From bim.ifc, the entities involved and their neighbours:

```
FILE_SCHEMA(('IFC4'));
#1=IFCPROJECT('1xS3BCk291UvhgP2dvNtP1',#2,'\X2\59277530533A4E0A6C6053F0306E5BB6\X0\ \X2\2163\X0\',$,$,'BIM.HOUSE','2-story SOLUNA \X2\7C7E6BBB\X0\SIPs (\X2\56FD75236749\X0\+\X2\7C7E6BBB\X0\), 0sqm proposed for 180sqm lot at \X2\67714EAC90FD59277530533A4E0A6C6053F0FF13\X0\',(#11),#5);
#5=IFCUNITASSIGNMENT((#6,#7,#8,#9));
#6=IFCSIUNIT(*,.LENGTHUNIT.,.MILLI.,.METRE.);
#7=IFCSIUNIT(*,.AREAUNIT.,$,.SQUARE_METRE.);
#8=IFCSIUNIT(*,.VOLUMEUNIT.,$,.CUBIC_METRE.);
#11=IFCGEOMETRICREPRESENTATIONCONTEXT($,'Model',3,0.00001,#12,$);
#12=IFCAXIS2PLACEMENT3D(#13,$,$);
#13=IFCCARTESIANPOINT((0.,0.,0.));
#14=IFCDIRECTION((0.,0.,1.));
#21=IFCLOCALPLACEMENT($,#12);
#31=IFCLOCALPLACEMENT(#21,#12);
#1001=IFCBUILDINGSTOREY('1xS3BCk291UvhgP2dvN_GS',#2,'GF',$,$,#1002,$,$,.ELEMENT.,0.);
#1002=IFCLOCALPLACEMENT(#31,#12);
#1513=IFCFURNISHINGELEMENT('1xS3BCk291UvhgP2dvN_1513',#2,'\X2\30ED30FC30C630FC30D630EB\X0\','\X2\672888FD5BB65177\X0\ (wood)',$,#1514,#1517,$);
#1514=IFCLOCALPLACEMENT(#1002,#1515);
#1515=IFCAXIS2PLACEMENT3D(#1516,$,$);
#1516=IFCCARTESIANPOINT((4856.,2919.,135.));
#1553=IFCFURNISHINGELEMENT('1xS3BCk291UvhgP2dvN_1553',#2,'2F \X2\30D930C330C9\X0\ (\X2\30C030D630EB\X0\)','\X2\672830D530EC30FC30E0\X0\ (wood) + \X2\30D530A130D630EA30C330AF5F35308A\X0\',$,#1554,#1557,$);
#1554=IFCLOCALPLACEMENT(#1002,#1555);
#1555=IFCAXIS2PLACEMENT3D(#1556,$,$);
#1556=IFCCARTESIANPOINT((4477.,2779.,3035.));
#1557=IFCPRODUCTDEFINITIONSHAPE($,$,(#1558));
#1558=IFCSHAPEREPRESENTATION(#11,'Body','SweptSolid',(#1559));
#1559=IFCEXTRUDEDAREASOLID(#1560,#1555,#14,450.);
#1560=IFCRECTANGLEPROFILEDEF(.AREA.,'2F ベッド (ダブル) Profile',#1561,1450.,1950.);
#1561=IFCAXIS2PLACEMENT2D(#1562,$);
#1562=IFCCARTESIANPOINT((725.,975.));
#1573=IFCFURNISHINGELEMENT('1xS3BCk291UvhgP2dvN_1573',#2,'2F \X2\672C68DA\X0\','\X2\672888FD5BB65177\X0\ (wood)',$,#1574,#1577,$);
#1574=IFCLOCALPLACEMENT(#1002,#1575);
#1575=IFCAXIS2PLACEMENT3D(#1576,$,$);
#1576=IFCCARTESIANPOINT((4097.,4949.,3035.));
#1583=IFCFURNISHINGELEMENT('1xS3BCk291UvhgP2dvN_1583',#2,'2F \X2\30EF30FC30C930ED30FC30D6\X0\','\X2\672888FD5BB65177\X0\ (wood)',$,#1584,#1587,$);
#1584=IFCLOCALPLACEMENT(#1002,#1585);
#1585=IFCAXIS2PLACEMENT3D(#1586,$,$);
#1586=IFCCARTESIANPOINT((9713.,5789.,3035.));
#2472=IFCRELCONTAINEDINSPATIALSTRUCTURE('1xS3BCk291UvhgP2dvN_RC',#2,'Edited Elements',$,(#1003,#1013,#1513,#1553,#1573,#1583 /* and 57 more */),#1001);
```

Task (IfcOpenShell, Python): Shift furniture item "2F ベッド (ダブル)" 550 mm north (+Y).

```python
import ifcopenshell
import ifcopenshell.api.geometry
import ifcopenshell.util.placement
import ifcopenshell.util.unit

model = ifcopenshell.open("bim.ifc")
unit_scale = ifcopenshell.util.unit.calculate_unit_scale(model)

item = model.by_guid("1xS3BCk291UvhgP2dvN_1553")
matrix = ifcopenshell.util.placement.get_local_placement(item.ObjectPlacement)
matrix[1, 3] += 0.55 / unit_scale
ifcopenshell.api.geometry.edit_object_placement(model, product=item, matrix=matrix, is_si=False)

print(ifcopenshell.util.placement.get_local_placement(item.ObjectPlacement).round(3) + 0.0)

model.write("bim_updated.ifc")
```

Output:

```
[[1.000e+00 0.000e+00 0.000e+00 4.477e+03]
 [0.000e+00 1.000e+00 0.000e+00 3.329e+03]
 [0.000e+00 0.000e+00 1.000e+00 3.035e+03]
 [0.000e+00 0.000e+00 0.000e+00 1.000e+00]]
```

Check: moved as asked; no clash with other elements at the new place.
